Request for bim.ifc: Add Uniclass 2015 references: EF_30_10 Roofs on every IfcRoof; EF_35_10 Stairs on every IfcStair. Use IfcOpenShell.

First a look at what the model holds.

```python
import ifcopenshell

model = ifcopenshell.open("bim.ifc")
print(model.schema)
print("classifications:", [c.Name for c in model.by_type("IfcClassification")])
for ifc_class in ("IfcDoor", "IfcRoof", "IfcStair", "IfcWall", "IfcWindow"):
    print(ifc_class, len(model.by_type(ifc_class)))
```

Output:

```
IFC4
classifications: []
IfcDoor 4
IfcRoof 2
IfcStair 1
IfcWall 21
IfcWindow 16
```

```python
import ifcopenshell
import ifcopenshell.api.classification

model = ifcopenshell.open("bim.ifc")

system = ifcopenshell.api.classification.add_classification(model, classification="Uniclass 2015")

codes = {
    "IfcRoof": ("EF_30_10", "Roofs"),
    "IfcStair": ("EF_35_10", "Stairs"),
}
for ifc_class, (code, name) in codes.items():
    products = model.by_type(ifc_class)
    ifcopenshell.api.classification.add_reference(
        model, products=products, classification=system, identification=code, name=name
    )
    print(code, len(products))

model.write("bim-out.ifc")
```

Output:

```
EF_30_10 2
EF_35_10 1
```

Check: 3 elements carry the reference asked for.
